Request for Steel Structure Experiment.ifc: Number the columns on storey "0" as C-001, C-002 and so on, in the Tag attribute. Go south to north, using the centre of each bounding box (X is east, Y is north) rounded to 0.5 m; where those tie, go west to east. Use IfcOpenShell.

First a look at what the model holds.

```python
import ifcopenshell
import ifcopenshell.util.element
import ifcopenshell.util.placement

model = ifcopenshell.open("Steel Structure Experiment.ifc")
print(model.schema)
storey = next(s for s in model.by_type("IfcBuildingStorey") if s.Name == "0")
columns = [e for e in ifcopenshell.util.element.get_decomposition(storey) if e.is_a("IfcColumn")]
for e in sorted(columns, key=lambda e: e.id()):
    origin = ifcopenshell.util.placement.get_local_placement(e.ObjectPlacement)[:3, 3]
    print(e.id(), e.Tag, e.Name, origin.round(2) + 0.0, sep=" | ")
```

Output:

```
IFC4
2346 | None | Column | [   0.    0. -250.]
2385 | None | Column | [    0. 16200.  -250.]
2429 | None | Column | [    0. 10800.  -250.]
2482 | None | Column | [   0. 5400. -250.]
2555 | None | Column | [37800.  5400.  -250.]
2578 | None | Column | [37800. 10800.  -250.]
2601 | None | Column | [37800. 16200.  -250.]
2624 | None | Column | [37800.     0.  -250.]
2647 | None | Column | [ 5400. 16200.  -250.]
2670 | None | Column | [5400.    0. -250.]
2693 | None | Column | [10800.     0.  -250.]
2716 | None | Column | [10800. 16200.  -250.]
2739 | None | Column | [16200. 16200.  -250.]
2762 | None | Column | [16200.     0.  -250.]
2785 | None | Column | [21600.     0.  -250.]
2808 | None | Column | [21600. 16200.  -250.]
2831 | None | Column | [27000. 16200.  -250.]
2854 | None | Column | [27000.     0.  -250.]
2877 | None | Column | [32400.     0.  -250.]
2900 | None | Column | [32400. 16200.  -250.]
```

```python
import ifcopenshell
import ifcopenshell.geom
import ifcopenshell.util.element
import ifcopenshell.util.shape

model = ifcopenshell.open("Steel Structure Experiment.ifc")
settings = ifcopenshell.geom.settings()
settings.set("use-world-coords", True)


def centre(element):
    shape = ifcopenshell.geom.create_shape(settings, element)
    return ifcopenshell.util.shape.get_bbox_centroid(shape.geometry)


storey = next(s for s in model.by_type("IfcBuildingStorey") if s.Name == "0")
columns = [e for e in ifcopenshell.util.element.get_decomposition(storey) if e.is_a("IfcColumn")]

# Insertion points can sit at a corner or the storey origin, so sort by the geometry (in metres).
centres = {e: centre(e) for e in columns}
columns.sort(key=lambda e: (round(centres[e][1] / 0.5), centres[e][0]))

for i, e in enumerate(columns, start=1):
    number = f"C-0{i:02d}"
    e.Tag = number
    print(e.id(), number)

model.write("Steel Structure Experiment_updated.ifc")
```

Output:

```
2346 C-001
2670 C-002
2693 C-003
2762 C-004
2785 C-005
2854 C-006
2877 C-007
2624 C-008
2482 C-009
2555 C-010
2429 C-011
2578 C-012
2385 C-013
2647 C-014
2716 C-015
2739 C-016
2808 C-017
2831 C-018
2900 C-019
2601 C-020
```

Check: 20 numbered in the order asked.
